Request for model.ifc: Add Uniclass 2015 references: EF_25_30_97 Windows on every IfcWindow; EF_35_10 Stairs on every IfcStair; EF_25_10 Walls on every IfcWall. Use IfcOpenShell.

First a look at what the model holds.

```python
import ifcopenshell

model = ifcopenshell.open("model.ifc")
print(model.schema)
print("classifications:", [c.Name for c in model.by_type("IfcClassification")])
for ifc_class in ("IfcDoor", "IfcRoof", "IfcStair", "IfcWall", "IfcWindow"):
    print(ifc_class, len(model.by_type(ifc_class)))
```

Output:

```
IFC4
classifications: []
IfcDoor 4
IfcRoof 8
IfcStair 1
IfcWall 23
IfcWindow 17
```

```python
import ifcopenshell
import ifcopenshell.api.classification

model = ifcopenshell.open("model.ifc")

system = ifcopenshell.api.classification.add_classification(model, classification="Uniclass 2015")

codes = {
    "IfcWindow": ("EF_25_30_97", "Windows"),
    "IfcStair": ("EF_35_10", "Stairs"),
    "IfcWall": ("EF_25_10", "Walls"),
}
for ifc_class, (code, name) in codes.items():
    products = model.by_type(ifc_class)
    ifcopenshell.api.classification.add_reference(
        model, products=products, classification=system, identification=code, name=name
    )
    print(code, len(products))

model.write("model_rev.ifc")
```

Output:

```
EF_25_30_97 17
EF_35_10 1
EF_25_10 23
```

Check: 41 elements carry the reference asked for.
